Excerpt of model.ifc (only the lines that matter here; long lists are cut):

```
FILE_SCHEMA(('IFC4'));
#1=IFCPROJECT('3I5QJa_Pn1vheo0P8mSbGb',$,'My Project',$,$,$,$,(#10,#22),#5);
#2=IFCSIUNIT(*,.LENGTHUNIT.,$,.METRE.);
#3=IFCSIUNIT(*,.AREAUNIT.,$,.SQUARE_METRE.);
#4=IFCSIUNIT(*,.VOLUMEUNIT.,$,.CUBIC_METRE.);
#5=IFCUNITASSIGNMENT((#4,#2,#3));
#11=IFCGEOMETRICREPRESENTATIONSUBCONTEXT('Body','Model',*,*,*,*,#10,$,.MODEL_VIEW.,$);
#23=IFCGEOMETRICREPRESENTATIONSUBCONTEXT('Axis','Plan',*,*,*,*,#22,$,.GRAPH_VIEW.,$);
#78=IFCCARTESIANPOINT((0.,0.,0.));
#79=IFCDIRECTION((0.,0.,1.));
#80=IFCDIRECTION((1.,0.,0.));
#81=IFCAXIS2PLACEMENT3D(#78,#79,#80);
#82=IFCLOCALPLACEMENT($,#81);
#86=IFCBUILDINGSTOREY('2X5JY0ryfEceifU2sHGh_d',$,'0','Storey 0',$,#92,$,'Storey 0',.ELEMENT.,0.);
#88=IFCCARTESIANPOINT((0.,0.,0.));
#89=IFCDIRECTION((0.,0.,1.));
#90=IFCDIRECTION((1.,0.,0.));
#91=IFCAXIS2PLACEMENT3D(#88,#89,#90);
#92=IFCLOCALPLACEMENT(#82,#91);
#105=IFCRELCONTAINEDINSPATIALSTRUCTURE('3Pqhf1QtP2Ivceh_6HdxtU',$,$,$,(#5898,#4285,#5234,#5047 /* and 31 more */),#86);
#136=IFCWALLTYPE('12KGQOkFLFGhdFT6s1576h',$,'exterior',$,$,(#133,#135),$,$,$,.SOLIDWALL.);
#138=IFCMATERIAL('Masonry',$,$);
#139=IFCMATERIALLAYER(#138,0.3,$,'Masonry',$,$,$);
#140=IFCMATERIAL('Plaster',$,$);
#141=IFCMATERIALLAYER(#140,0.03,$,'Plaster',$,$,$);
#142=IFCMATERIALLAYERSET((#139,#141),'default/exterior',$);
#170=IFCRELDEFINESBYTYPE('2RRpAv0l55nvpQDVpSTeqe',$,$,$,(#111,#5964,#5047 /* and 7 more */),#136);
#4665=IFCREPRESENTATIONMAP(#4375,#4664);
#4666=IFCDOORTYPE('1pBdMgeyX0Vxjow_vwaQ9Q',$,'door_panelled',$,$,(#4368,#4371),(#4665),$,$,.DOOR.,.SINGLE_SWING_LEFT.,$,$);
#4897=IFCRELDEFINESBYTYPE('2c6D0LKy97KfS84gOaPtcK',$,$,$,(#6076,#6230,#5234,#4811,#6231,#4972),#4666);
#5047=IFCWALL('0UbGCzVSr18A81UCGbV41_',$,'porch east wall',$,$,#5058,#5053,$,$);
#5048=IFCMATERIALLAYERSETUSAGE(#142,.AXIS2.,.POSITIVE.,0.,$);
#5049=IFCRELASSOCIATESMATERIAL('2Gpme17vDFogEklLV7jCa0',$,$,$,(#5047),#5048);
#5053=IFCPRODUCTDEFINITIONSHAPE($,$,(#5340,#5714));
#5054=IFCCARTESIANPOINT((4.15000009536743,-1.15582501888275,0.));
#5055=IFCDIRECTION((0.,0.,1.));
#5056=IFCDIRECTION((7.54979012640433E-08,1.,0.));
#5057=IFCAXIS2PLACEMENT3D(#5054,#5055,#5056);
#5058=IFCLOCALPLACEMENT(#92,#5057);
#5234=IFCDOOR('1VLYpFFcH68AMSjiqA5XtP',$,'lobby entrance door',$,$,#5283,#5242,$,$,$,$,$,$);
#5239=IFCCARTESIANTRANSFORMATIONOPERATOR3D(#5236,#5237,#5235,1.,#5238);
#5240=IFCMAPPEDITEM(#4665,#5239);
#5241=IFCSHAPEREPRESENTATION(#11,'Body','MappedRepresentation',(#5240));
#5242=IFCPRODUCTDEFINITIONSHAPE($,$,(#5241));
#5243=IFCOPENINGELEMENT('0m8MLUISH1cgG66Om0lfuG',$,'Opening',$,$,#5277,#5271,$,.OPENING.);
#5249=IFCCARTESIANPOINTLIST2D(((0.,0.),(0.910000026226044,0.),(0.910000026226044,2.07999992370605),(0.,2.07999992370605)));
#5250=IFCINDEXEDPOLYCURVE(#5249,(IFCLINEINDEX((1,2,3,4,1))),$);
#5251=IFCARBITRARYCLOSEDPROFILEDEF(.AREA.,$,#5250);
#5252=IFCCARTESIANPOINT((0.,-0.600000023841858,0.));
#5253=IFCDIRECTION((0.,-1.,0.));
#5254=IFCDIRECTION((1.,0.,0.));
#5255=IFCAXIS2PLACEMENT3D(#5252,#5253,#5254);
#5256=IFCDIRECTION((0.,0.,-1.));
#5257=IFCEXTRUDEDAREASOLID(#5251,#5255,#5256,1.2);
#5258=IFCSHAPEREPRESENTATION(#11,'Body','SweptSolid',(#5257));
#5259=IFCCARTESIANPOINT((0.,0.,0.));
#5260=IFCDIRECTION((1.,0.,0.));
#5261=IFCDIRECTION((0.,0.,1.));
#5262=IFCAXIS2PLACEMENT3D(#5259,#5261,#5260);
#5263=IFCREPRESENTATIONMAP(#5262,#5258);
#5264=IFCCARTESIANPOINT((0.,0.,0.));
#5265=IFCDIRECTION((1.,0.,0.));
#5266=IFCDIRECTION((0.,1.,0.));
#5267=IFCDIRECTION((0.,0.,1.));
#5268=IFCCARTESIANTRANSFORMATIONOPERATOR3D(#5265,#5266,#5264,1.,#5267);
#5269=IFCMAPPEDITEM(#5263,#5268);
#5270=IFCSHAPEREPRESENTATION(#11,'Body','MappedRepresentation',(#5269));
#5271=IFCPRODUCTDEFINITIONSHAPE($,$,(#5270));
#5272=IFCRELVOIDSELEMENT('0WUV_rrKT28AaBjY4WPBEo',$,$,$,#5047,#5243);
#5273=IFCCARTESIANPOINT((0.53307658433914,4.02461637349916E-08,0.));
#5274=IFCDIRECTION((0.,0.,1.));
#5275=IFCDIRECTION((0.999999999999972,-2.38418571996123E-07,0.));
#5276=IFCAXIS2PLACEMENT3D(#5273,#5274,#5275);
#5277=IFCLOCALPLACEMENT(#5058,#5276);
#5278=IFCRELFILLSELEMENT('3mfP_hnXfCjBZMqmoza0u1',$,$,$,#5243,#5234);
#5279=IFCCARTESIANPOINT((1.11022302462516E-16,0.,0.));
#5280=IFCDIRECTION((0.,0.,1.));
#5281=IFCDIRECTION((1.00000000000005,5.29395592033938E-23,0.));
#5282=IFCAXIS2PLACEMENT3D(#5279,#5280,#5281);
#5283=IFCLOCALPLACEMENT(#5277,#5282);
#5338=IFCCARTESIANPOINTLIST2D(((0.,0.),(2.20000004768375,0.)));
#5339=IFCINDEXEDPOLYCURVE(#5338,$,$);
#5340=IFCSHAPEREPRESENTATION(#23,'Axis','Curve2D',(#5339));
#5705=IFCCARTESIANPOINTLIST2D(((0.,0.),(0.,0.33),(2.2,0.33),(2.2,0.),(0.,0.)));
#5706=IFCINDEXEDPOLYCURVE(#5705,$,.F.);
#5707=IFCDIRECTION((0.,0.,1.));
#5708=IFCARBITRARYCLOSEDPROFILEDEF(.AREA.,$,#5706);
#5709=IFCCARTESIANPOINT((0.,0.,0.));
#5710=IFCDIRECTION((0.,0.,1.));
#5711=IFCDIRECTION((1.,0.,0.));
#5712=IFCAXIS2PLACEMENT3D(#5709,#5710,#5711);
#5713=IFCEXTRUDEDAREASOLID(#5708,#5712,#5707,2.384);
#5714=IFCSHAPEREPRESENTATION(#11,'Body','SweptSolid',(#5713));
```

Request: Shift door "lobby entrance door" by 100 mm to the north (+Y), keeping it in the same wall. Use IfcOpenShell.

```python
import ifcopenshell
import ifcopenshell.api.geometry
import ifcopenshell.util.placement

model = ifcopenshell.open("model.ifc")

door = model.by_guid("1VLYpFFcH68AMSjiqA5XtP")
opening = door.FillsVoids[0].RelatingOpeningElement
wall = opening.VoidsElements[0].RelatingBuildingElement

wall_matrix = ifcopenshell.util.placement.get_local_placement(wall.ObjectPlacement)
shift = wall_matrix[:3, 0] * 0.1
before = ifcopenshell.util.placement.get_local_placement(door.ObjectPlacement)[:3, 3].copy()

# The door is placed relative to its opening, so it follows when the opening moves.
matrix = ifcopenshell.util.placement.get_local_placement(opening.ObjectPlacement)
matrix[:3, 3] += shift
ifcopenshell.api.geometry.edit_object_placement(
    model, product=opening, matrix=matrix, is_si=False, should_transform_children=True
)

after = ifcopenshell.util.placement.get_local_placement(door.ObjectPlacement)[:3, 3]
print("door moved by", (after - before).round(3) + 0.0)

model.write("model_rev.ifc")
```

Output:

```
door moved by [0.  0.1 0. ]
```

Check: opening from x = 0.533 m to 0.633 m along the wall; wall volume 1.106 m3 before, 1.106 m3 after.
